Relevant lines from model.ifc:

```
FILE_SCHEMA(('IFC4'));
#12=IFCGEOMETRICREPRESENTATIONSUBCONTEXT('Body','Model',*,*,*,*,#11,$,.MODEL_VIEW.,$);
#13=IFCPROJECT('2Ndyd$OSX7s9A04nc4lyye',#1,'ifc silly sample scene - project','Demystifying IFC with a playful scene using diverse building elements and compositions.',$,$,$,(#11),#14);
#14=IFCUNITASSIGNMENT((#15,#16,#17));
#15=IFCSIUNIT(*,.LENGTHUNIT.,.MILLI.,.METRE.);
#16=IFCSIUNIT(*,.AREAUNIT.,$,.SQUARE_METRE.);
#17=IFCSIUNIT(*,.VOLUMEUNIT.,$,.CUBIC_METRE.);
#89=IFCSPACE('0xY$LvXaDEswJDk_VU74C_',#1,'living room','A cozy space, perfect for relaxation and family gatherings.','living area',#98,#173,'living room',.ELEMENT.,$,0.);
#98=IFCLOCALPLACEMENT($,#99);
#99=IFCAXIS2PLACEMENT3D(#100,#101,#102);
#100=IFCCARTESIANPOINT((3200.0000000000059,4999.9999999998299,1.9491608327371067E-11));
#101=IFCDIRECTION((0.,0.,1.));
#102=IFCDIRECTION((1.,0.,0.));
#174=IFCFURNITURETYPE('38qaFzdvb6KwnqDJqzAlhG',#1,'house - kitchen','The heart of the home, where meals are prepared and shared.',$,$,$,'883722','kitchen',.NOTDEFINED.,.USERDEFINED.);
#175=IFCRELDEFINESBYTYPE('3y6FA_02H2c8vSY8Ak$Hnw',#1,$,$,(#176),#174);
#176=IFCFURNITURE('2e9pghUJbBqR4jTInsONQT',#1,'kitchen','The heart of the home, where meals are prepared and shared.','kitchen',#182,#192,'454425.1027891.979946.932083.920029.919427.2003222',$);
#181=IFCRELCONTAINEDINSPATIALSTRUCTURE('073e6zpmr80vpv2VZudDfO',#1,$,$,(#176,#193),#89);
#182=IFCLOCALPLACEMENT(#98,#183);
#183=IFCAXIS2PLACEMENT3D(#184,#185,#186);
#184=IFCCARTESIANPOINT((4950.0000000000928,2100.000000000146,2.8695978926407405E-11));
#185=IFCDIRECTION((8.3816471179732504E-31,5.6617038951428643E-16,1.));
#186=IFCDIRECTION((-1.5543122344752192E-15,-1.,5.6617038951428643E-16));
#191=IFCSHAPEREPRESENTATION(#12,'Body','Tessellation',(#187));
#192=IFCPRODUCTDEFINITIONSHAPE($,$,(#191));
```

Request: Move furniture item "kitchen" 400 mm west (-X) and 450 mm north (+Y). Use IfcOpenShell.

```python
import ifcopenshell
import ifcopenshell.api.geometry
import ifcopenshell.util.placement
import ifcopenshell.util.unit

model = ifcopenshell.open("model.ifc")
unit_scale = ifcopenshell.util.unit.calculate_unit_scale(model)

item = model.by_id(176)
matrix = ifcopenshell.util.placement.get_local_placement(item.ObjectPlacement)
matrix[0, 3] -= 0.4 / unit_scale
matrix[1, 3] += 0.45 / unit_scale
ifcopenshell.api.geometry.edit_object_placement(model, product=item, matrix=matrix, is_si=False)

print(ifcopenshell.util.placement.get_local_placement(item.ObjectPlacement).round(3) + 0.0)

model.write("model_v2.ifc")
```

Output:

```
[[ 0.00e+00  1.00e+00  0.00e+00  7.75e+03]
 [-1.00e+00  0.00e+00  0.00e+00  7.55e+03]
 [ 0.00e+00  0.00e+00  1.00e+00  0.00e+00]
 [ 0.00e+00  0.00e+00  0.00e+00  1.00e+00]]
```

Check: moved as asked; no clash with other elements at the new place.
